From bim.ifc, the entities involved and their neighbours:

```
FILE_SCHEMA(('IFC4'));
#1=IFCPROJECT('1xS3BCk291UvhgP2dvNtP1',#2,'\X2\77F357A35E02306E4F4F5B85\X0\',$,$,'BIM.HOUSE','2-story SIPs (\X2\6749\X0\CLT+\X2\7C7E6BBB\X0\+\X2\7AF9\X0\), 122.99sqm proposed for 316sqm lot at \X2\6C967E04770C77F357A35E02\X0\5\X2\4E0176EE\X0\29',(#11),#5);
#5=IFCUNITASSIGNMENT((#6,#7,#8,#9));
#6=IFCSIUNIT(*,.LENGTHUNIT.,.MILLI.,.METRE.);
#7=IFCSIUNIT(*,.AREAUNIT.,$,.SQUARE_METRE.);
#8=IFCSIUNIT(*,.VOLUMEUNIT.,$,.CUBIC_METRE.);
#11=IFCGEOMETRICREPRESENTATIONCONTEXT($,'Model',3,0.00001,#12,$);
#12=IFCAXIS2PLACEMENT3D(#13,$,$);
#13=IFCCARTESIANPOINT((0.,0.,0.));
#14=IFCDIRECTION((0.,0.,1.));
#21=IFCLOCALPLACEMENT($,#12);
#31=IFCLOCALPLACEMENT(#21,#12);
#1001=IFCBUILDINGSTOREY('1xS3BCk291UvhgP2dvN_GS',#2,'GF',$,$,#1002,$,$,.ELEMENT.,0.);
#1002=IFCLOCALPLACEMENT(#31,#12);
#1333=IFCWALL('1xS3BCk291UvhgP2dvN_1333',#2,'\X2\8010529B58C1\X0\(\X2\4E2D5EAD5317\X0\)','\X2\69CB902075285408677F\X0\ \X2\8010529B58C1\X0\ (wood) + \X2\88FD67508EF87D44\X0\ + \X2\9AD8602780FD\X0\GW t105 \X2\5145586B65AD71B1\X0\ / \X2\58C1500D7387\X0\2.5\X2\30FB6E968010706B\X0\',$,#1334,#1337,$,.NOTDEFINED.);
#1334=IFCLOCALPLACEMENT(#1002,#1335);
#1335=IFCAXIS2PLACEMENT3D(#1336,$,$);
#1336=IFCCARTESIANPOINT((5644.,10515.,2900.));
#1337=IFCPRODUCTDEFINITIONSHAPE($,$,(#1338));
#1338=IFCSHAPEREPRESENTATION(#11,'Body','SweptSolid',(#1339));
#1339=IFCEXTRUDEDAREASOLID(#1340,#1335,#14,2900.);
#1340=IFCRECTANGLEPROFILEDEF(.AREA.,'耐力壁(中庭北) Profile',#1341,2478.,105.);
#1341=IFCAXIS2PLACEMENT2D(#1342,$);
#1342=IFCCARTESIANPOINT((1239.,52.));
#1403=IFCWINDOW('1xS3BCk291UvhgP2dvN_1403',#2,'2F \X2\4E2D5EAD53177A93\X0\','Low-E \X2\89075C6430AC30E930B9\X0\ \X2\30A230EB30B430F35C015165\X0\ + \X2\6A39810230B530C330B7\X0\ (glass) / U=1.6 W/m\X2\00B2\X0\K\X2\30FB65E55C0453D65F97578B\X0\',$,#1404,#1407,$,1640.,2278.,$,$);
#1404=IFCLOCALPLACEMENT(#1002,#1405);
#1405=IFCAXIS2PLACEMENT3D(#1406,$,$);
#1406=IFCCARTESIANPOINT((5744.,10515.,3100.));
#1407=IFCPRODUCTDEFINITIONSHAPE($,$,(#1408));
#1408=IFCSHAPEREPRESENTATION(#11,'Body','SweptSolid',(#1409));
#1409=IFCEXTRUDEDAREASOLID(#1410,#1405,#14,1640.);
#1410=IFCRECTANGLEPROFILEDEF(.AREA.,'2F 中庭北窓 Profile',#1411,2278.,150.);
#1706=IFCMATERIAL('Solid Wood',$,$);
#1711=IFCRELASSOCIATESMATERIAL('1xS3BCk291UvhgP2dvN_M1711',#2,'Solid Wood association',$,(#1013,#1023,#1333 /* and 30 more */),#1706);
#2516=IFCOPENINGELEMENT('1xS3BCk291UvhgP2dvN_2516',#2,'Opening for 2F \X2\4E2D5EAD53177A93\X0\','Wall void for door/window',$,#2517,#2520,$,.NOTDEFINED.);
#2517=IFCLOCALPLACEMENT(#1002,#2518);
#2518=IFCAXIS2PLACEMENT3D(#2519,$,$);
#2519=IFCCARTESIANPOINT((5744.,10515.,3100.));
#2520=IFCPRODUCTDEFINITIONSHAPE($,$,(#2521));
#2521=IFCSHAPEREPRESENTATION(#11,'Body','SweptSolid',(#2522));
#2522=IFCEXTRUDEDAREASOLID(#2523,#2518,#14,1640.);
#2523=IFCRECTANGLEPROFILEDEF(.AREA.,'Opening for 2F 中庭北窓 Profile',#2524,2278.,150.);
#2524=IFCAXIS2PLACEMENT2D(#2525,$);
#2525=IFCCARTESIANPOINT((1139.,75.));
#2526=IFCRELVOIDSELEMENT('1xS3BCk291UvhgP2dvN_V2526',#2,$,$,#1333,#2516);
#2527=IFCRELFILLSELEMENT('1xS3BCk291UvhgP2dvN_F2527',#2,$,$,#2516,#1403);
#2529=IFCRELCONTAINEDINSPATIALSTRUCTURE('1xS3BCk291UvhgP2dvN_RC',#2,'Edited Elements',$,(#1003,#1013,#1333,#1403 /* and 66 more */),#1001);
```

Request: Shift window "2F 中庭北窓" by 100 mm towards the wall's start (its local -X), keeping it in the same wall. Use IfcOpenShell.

```python
import ifcopenshell
import ifcopenshell.api.geometry
import ifcopenshell.util.placement
import ifcopenshell.util.unit

model = ifcopenshell.open("bim.ifc")
unit_scale = ifcopenshell.util.unit.calculate_unit_scale(model)

window = model.by_guid("1xS3BCk291UvhgP2dvN_1403")
opening = window.FillsVoids[0].RelatingOpeningElement
wall = opening.VoidsElements[0].RelatingBuildingElement

wall_matrix = ifcopenshell.util.placement.get_local_placement(wall.ObjectPlacement)
shift = wall_matrix[:3, 0] * -0.1 / unit_scale
before = ifcopenshell.util.placement.get_local_placement(window.ObjectPlacement)[:3, 3].copy()

# The window is not placed relative to its opening, so move both.
for product in (opening, window):
    matrix = ifcopenshell.util.placement.get_local_placement(product.ObjectPlacement)
    matrix[:3, 3] += shift
    ifcopenshell.api.geometry.edit_object_placement(model, product=product, matrix=matrix, is_si=False)

after = ifcopenshell.util.placement.get_local_placement(window.ObjectPlacement)[:3, 3]
print("window moved by", (after - before).round(3) + 0.0)

model.write("bim_updated.ifc")
```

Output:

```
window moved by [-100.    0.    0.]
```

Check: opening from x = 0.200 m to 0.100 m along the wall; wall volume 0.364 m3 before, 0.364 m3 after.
